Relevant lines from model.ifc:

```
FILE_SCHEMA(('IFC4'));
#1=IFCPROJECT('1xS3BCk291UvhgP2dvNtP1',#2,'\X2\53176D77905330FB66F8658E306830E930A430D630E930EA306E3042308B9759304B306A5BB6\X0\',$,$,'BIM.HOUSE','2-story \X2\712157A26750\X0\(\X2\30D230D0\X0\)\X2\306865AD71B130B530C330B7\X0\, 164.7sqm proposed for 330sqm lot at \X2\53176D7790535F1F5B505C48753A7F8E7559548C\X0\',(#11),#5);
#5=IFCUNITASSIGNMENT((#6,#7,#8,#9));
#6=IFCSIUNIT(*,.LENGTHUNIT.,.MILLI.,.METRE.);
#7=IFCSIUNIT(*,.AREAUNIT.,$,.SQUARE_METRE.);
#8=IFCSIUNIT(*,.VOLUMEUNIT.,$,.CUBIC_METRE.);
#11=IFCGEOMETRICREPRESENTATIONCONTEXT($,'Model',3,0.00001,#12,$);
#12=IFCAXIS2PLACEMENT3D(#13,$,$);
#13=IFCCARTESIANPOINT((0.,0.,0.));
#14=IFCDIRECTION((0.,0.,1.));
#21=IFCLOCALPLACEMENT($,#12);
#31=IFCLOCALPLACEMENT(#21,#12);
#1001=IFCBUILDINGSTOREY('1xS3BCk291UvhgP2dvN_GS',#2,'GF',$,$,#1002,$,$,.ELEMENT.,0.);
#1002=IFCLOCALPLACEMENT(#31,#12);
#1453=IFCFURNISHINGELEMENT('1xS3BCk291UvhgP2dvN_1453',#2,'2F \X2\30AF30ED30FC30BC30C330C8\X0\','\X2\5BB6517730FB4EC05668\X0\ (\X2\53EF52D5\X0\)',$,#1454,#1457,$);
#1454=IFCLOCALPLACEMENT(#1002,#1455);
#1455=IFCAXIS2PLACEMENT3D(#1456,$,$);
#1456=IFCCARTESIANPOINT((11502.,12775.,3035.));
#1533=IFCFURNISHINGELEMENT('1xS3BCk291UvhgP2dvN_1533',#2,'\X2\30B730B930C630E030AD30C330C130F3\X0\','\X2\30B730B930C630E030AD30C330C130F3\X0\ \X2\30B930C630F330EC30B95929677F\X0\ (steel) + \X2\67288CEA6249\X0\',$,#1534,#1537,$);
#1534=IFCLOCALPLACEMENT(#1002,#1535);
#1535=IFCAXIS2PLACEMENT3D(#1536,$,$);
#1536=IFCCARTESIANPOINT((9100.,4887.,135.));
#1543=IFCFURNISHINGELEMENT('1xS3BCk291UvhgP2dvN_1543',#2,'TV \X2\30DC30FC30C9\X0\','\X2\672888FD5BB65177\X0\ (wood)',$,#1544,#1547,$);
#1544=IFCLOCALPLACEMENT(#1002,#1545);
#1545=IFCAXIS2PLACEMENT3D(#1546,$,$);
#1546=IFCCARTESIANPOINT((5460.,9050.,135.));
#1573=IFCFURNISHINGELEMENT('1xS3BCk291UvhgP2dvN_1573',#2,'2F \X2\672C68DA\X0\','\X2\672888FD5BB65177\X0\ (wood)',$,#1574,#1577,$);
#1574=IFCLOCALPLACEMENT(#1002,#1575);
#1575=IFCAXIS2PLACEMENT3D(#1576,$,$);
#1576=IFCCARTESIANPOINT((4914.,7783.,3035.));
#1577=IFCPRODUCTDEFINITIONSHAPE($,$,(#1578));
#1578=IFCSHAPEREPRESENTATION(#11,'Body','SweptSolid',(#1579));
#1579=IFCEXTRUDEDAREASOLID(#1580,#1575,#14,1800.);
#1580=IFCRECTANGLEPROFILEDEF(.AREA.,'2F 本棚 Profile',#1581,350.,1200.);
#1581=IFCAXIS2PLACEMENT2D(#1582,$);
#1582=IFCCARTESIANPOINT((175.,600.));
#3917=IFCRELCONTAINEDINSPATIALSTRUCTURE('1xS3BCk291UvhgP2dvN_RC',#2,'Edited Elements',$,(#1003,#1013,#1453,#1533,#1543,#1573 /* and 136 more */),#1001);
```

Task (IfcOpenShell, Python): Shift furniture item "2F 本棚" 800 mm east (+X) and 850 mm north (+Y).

```python
import ifcopenshell
import ifcopenshell.api.geometry
import ifcopenshell.util.placement
import ifcopenshell.util.unit

model = ifcopenshell.open("model.ifc")
unit_scale = ifcopenshell.util.unit.calculate_unit_scale(model)

item = model.by_guid("1xS3BCk291UvhgP2dvN_1573")
matrix = ifcopenshell.util.placement.get_local_placement(item.ObjectPlacement)
matrix[0, 3] += 0.8 / unit_scale
matrix[1, 3] += 0.85 / unit_scale
ifcopenshell.api.geometry.edit_object_placement(model, product=item, matrix=matrix, is_si=False)

print(ifcopenshell.util.placement.get_local_placement(item.ObjectPlacement).round(3) + 0.0)

model.write("model_rev.ifc")
```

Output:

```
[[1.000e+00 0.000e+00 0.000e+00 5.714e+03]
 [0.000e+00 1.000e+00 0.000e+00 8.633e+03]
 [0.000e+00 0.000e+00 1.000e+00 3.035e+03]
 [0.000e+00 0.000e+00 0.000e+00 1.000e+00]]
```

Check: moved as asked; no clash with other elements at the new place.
